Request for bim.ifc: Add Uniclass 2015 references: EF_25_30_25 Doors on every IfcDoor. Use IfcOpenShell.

First a look at what the model holds.

```python
import ifcopenshell

model = ifcopenshell.open("bim.ifc")
print(model.schema)
print("classifications:", [c.Name for c in model.by_type("IfcClassification")])
for ifc_class in ("IfcDoor", "IfcRoof", "IfcStair", "IfcWall", "IfcWindow"):
    print(ifc_class, len(model.by_type(ifc_class)))
```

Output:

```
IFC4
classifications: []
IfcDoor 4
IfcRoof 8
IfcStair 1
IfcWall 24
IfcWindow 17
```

```python
import ifcopenshell
import ifcopenshell.api.classification

model = ifcopenshell.open("bim.ifc")

system = ifcopenshell.api.classification.add_classification(model, classification="Uniclass 2015")

codes = {
    "IfcDoor": ("EF_25_30_25", "Doors"),
}
for ifc_class, (code, name) in codes.items():
    products = model.by_type(ifc_class)
    ifcopenshell.api.classification.add_reference(
        model, products=products, classification=system, identification=code, name=name
    )
    print(code, len(products))

model.write("bim_edited.ifc")
```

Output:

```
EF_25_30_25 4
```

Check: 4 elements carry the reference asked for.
